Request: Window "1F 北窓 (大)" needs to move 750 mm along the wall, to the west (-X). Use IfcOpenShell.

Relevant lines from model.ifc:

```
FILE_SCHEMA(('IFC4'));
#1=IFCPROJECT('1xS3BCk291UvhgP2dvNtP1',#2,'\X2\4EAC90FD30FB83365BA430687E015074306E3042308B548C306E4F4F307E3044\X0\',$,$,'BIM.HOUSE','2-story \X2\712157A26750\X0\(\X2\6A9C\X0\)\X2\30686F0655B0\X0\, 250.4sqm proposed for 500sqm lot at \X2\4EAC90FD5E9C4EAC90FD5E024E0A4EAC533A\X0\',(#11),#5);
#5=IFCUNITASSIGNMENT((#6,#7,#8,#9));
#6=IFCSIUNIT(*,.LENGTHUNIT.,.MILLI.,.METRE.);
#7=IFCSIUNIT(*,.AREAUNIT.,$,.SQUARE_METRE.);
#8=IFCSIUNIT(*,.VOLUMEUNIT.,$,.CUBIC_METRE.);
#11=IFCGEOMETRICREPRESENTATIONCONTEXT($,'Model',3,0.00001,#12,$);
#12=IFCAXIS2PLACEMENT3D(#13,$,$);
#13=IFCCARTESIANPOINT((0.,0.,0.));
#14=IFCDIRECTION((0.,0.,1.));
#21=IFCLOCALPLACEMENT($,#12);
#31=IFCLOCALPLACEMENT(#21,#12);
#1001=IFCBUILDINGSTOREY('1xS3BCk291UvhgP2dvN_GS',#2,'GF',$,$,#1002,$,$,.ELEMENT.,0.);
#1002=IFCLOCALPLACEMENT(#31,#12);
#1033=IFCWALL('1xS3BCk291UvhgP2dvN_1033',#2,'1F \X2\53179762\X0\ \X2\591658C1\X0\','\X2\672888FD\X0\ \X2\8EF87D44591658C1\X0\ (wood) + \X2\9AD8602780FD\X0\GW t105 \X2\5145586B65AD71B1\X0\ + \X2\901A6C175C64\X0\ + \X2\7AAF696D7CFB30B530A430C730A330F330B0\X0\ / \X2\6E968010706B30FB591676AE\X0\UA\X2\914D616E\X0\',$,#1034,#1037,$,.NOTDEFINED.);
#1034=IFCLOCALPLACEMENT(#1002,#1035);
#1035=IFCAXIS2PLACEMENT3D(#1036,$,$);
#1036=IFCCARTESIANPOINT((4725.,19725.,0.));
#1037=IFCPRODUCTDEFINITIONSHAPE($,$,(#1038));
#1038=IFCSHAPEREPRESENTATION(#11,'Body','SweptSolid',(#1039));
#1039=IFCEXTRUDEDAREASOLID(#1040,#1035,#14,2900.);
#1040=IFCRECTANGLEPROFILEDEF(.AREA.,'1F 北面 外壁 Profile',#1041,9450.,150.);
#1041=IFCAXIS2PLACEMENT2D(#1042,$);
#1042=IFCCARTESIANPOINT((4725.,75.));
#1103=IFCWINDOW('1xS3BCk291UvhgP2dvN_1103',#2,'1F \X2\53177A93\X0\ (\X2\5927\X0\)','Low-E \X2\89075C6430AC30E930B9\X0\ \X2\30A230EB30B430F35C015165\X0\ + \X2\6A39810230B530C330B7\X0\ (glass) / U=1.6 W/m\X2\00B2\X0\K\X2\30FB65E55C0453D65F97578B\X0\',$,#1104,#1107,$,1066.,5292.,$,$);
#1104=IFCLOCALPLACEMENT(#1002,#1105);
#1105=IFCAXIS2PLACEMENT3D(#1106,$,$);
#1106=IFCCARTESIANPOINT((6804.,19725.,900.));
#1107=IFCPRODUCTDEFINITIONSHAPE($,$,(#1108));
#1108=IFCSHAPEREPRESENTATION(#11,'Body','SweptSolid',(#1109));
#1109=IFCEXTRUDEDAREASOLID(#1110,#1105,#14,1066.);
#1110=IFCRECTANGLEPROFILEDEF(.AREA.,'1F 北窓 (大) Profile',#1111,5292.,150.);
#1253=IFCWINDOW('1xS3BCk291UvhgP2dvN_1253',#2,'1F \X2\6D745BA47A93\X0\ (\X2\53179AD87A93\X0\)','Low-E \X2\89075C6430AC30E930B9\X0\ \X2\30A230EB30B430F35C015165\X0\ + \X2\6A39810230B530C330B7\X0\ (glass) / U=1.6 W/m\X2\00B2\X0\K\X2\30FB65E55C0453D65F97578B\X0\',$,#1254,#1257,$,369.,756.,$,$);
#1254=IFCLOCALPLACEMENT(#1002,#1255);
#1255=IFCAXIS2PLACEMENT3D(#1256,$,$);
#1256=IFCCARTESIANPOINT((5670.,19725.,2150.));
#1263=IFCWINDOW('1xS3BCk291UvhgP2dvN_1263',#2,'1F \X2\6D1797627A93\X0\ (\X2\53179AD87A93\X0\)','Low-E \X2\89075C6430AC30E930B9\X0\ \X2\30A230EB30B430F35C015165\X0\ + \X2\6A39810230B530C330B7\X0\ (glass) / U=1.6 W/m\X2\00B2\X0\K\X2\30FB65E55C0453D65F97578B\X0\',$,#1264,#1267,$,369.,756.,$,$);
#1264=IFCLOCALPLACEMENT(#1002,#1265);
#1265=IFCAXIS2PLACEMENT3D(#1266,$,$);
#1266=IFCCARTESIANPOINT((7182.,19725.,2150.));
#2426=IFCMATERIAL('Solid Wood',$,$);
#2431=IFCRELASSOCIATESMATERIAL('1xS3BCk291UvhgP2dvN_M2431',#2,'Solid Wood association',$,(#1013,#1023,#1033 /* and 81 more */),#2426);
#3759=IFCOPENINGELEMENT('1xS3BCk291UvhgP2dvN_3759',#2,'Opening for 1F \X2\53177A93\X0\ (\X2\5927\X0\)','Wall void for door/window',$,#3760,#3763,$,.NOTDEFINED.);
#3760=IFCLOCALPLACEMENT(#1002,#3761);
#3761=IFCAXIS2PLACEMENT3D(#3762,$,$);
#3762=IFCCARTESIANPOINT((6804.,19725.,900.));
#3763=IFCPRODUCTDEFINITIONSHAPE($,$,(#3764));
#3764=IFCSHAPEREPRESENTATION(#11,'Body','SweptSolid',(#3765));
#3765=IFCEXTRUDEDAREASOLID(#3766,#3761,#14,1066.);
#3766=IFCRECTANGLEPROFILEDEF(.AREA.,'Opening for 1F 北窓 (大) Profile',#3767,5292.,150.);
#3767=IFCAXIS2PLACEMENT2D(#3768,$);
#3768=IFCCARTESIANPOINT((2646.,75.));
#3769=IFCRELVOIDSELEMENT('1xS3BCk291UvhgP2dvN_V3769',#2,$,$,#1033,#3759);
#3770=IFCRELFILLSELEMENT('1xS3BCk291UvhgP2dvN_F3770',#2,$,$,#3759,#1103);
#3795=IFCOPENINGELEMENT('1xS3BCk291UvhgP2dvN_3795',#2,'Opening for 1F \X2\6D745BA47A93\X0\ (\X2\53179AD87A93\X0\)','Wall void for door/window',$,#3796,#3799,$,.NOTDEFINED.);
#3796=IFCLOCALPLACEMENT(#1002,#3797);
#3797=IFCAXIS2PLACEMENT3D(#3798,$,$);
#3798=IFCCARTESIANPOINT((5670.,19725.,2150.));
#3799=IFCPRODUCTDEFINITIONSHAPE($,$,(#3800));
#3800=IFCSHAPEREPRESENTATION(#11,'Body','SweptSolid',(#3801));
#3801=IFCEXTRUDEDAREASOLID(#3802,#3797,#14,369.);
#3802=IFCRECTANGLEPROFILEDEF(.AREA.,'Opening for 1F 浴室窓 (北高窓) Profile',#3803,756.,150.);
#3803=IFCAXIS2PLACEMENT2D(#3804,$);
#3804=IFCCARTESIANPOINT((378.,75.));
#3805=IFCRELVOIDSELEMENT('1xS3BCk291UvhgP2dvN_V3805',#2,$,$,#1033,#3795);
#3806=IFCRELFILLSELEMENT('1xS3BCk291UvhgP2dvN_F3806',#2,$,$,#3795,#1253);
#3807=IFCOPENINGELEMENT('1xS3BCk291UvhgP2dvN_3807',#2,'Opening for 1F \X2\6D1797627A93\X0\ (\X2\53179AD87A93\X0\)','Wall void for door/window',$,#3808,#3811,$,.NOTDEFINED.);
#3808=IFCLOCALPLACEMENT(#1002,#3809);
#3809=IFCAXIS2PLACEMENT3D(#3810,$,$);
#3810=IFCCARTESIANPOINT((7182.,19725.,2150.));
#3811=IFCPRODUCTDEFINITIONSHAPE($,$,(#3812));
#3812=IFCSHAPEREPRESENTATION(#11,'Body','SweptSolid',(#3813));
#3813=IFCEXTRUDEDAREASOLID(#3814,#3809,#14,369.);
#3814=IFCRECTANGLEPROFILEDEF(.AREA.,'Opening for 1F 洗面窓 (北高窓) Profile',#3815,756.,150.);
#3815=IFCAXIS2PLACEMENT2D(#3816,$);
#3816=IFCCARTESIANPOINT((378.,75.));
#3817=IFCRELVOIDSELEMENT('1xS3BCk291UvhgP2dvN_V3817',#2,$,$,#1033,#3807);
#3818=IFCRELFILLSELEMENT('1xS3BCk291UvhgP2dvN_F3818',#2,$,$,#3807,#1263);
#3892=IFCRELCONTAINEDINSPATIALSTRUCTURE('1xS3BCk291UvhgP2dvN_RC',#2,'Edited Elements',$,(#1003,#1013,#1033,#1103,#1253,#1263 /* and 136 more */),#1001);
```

```python
import ifcopenshell
import ifcopenshell.api.geometry
import ifcopenshell.util.placement

model = ifcopenshell.open("model.ifc")

window = model.by_id(1103)
opening = window.FillsVoids[0].RelatingOpeningElement
wall = opening.VoidsElements[0].RelatingBuildingElement

wall_matrix = ifcopenshell.util.placement.get_local_placement(wall.ObjectPlacement)
shift = wall_matrix[:3, 0] * -750.0
before = ifcopenshell.util.placement.get_local_placement(window.ObjectPlacement)[:3, 3].copy()

# The window is not placed relative to its opening, so move both.
for product in (opening, window):
    matrix = ifcopenshell.util.placement.get_local_placement(product.ObjectPlacement)
    matrix[:3, 3] += shift
    ifcopenshell.api.geometry.edit_object_placement(model, product=product, matrix=matrix, is_si=False)

after = ifcopenshell.util.placement.get_local_placement(window.ObjectPlacement)[:3, 3]
print("window moved by", (after - before).round(3) + 0.0)

model.write("model_v2.ifc")
```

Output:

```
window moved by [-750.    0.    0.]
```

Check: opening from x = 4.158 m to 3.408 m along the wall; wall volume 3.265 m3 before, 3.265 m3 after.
